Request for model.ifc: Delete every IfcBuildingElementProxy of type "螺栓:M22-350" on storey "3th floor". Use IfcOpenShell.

First a look at what the model holds.

```python
import ifcopenshell
import ifcopenshell.util.element

model = ifcopenshell.open("model.ifc")
print(model.schema)
storey = next(s for s in model.by_type("IfcBuildingStorey") if s.Name == "3th floor")
proxies = [e for e in ifcopenshell.util.element.get_decomposition(storey) if e.is_a("IfcBuildingElementProxy")]
seen = {}
for e in proxies:
    element_type = ifcopenshell.util.element.get_type(e)
    name = element_type.Name if element_type not in (None, e) else None
    seen[name] = seen.get(name, 0) + 1
for name, count in sorted(seen.items(), key=str):
    print(count, "x", name)
```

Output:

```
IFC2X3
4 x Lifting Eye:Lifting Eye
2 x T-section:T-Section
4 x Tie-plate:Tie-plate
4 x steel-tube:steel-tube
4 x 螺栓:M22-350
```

```python
import ifcopenshell
import ifcopenshell.api.root
import ifcopenshell.util.element

model = ifcopenshell.open("model.ifc")

storey = next(s for s in model.by_type("IfcBuildingStorey") if s.Name == "3th floor")
proxies = [e for e in ifcopenshell.util.element.get_decomposition(storey) if e.is_a("IfcBuildingElementProxy")]
targets = [e for e in proxies if (t := ifcopenshell.util.element.get_type(e)) not in (None, e) and t.Name == "螺栓:M22-350"]

for e in targets:
    ifcopenshell.api.root.remove_product(model, product=e)
print(len(targets), "removed")

model.write("model-out.ifc")
```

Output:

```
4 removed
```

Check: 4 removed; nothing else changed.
